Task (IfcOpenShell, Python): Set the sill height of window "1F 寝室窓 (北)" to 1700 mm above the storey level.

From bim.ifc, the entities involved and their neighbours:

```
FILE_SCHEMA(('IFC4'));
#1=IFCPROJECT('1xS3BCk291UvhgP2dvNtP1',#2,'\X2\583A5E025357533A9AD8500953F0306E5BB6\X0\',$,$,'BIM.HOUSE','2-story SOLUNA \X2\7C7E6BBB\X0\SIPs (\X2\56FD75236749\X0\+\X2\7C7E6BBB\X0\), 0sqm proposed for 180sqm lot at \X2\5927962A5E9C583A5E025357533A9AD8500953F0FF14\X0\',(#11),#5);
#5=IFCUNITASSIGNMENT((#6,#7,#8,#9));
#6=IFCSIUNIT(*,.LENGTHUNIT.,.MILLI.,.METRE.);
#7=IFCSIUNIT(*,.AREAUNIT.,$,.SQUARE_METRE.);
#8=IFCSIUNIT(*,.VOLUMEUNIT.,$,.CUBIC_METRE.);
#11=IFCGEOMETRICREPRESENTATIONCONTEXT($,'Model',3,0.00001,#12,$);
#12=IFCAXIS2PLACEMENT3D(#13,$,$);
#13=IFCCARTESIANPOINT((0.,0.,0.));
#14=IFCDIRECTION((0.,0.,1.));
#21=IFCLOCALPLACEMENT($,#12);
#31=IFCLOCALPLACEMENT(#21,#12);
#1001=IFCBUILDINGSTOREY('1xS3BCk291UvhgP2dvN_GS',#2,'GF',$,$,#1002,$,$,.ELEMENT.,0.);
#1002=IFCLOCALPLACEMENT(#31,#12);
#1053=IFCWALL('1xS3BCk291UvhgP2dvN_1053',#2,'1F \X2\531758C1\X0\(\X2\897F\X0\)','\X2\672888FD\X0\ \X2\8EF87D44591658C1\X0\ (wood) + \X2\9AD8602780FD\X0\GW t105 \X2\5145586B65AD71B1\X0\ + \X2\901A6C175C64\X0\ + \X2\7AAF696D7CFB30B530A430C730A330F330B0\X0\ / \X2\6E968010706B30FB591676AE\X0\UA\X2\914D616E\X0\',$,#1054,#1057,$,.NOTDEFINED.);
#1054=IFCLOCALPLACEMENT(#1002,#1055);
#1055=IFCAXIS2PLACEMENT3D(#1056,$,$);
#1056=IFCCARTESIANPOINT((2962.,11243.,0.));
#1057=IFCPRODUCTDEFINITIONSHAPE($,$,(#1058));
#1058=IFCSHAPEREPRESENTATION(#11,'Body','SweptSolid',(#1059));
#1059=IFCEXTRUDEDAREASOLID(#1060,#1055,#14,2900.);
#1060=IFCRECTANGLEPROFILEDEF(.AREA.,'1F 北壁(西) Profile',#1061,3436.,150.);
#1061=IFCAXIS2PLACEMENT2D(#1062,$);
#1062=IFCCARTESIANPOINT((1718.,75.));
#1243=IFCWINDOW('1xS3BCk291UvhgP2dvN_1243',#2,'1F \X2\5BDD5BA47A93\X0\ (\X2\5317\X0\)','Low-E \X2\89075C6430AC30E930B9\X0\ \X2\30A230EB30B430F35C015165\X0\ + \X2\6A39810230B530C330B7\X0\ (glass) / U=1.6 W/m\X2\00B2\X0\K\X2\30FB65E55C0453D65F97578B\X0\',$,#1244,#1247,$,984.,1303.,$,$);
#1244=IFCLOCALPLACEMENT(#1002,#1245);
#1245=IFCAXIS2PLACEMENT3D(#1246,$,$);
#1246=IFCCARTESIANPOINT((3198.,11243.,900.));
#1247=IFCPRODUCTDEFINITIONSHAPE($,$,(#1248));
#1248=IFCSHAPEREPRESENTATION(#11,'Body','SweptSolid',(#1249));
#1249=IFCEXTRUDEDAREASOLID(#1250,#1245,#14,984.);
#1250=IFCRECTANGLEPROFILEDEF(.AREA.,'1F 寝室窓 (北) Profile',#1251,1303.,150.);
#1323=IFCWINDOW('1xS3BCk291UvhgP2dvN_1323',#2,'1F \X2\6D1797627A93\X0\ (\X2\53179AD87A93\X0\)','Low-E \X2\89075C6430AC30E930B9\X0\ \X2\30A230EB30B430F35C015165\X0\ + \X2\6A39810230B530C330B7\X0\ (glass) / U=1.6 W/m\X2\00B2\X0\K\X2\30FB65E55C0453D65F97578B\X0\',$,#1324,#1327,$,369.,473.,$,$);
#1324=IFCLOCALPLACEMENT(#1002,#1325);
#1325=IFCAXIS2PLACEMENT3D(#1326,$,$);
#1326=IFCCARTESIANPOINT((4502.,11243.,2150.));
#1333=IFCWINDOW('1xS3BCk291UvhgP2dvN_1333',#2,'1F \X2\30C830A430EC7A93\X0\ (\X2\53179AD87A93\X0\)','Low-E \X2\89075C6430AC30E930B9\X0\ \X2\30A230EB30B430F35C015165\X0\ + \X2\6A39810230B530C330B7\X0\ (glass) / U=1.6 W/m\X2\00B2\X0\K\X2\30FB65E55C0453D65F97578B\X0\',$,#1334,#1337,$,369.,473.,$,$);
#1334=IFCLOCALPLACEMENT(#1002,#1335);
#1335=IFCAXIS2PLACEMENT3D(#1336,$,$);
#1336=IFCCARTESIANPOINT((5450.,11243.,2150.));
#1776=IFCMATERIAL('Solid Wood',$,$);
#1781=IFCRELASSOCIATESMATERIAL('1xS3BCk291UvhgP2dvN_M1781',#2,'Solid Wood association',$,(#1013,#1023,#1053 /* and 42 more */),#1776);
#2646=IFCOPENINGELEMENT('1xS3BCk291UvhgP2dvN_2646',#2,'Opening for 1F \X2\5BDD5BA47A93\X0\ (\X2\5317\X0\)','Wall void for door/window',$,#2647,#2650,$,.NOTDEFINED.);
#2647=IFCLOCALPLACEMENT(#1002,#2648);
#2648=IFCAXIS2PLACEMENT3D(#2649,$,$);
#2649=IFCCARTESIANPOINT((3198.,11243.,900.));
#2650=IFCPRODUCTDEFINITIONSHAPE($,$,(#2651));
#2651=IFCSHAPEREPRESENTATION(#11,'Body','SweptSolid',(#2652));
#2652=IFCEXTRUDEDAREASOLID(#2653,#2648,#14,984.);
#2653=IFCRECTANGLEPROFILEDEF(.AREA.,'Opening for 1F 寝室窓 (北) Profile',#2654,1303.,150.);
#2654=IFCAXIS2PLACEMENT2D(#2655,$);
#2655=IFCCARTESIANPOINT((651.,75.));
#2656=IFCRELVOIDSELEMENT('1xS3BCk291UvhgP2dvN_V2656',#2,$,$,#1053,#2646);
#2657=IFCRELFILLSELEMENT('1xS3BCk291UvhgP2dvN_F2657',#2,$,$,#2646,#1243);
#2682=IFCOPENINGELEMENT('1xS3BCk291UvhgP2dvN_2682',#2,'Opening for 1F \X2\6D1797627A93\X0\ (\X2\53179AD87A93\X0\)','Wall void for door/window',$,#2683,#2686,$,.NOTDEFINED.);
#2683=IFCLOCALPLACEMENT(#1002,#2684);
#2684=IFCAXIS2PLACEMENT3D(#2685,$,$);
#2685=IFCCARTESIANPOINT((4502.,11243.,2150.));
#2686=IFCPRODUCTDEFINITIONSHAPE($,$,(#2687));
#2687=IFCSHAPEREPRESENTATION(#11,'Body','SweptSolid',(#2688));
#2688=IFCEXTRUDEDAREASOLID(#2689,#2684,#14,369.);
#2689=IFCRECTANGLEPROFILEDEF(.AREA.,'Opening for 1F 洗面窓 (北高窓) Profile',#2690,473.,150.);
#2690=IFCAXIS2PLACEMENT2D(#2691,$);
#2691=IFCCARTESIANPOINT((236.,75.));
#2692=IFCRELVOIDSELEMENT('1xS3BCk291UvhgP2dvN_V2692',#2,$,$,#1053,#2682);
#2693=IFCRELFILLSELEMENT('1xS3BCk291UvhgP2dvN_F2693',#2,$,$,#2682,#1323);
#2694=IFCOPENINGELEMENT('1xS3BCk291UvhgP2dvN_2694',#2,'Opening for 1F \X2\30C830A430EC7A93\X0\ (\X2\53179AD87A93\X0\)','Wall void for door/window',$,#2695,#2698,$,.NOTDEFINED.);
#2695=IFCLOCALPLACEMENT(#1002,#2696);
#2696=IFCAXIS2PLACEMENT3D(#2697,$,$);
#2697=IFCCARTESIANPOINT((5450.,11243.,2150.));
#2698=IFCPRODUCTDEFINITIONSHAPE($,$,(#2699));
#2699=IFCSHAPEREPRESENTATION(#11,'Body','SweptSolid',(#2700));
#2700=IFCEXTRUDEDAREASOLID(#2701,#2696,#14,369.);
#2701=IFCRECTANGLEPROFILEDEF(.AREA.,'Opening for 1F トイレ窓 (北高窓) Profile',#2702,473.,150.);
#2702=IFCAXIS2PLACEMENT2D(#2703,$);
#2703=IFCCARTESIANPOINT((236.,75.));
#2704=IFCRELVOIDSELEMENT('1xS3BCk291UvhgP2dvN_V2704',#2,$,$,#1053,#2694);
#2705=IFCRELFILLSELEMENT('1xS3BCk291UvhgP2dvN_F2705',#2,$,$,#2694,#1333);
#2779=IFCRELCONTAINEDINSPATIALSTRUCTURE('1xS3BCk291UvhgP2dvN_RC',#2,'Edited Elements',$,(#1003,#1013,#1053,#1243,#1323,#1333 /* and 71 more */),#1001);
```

```python
import numpy as np
import ifcopenshell
import ifcopenshell.api.geometry
import ifcopenshell.geom
import ifcopenshell.util.element
import ifcopenshell.util.placement
import ifcopenshell.util.shape
import ifcopenshell.util.unit

model = ifcopenshell.open("bim.ifc")
unit_scale = ifcopenshell.util.unit.calculate_unit_scale(model)

window = model.by_guid("1xS3BCk291UvhgP2dvN_1243")
opening = window.FillsVoids[0].RelatingOpeningElement
storey = ifcopenshell.util.element.get_container(window, ifc_class="IfcBuildingStorey")
level = ifcopenshell.util.placement.get_local_placement(storey.ObjectPlacement)[2, 3]

# The opening's origin need not be at the sill, so measure its lowest point.
shape = ifcopenshell.geom.create_shape(ifcopenshell.geom.settings(), opening)
bottom = ifcopenshell.util.shape.get_shape_bottom_elevation(shape, shape.geometry) / unit_scale
dz = level + 1.7 / unit_scale - bottom

shift = np.array([0.0, 0.0, dz])
# The window is not placed relative to its opening, so move both.
for product in (opening, window):
    matrix = ifcopenshell.util.placement.get_local_placement(product.ObjectPlacement)
    matrix[:3, 3] += shift
    ifcopenshell.api.geometry.edit_object_placement(model, product=product, matrix=matrix, is_si=False)

print(f"moved by {dz * unit_scale:+.3f} m")

model.write("bim_edited.ifc")
```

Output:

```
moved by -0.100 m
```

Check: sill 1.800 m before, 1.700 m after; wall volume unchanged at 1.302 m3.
